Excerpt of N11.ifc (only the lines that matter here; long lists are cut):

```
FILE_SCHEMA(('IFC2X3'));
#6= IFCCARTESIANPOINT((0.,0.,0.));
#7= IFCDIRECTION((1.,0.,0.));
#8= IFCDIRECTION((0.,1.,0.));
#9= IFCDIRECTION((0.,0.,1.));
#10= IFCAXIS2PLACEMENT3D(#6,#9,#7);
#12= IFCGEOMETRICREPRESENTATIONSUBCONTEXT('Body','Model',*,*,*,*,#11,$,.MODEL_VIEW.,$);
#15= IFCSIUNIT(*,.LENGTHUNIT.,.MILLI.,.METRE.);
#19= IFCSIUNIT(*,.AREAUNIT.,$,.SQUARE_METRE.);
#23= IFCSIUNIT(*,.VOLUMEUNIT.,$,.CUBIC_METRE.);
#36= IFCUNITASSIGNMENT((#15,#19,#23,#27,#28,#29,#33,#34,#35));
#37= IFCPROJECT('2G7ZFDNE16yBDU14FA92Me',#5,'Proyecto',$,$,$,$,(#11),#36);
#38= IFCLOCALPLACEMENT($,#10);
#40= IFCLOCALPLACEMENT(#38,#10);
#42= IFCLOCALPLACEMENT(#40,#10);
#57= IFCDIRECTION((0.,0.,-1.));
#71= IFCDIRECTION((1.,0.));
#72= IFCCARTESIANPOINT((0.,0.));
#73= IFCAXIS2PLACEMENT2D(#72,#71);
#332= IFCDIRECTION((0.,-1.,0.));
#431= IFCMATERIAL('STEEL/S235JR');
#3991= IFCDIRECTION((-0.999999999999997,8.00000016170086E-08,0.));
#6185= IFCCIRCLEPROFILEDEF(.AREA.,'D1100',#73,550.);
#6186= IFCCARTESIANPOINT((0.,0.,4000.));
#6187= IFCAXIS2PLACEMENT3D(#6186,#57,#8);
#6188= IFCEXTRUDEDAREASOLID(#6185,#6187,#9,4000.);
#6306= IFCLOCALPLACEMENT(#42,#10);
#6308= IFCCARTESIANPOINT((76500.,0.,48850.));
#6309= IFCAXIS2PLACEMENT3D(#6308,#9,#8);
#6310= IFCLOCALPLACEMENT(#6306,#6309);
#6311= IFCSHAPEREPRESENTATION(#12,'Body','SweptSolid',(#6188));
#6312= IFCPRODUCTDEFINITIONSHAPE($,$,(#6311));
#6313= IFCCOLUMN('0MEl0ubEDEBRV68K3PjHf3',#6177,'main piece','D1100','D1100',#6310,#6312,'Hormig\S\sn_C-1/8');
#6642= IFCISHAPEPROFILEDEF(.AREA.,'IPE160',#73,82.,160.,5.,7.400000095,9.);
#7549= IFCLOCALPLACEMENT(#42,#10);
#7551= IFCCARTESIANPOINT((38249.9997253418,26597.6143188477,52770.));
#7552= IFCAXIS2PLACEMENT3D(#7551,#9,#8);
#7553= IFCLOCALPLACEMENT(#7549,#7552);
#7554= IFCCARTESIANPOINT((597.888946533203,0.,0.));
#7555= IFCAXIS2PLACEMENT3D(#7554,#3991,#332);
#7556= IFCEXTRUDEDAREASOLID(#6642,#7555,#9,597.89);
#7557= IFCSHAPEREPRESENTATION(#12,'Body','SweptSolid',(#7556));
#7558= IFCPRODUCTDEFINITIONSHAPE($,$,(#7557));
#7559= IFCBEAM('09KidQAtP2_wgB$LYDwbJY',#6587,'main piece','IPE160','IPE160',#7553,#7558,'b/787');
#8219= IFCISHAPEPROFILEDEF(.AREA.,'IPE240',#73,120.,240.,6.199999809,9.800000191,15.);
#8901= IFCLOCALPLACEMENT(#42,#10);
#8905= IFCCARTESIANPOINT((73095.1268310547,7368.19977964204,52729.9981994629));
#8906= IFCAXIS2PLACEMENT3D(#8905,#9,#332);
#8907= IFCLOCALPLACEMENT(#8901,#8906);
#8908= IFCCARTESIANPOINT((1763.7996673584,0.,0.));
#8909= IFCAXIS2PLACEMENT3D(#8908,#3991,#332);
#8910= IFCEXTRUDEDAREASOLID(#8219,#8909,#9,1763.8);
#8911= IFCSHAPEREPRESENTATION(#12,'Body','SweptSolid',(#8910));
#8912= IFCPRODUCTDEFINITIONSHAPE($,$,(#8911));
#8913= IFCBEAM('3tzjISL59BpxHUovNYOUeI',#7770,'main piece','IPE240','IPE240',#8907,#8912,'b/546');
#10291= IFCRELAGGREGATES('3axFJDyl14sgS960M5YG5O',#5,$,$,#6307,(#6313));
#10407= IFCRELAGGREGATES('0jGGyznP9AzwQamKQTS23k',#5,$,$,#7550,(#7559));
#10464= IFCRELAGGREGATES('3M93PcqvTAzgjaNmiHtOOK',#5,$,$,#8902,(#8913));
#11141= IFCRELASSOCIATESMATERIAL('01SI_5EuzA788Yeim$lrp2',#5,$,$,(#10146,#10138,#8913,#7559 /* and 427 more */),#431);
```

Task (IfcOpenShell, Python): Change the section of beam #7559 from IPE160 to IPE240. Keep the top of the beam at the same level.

```python
import ifcopenshell
import ifcopenshell.util.element
import ifcopenshell.util.representation

model = ifcopenshell.open("N11.ifc")

member = model.by_id(7559)
source = next(p for p in model.by_type("IfcIShapeProfileDef") if p.ProfileName == "IPE240")

body = ifcopenshell.util.representation.get_representation(member, "Model", "Body")
solid = body.Items[0]
old_profile = solid.SweptArea

# Copy the section's sizes but keep this member's own profile position.
profile = ifcopenshell.util.element.copy(model, source)
# Profiles are centred, so shift by half the change in depth to hold the top.
shift = (old_profile.OverallDepth - profile.OverallDepth) / 2
x, y = old_profile.Position.Location.Coordinates
up = (0.0, 1.0)  # upwards, in the solid's own plane
location = model.createIfcCartesianPoint((x + up[0] * shift, y + up[1] * shift))
profile.Position = model.createIfcAxis2Placement2D(location, old_profile.Position.RefDirection)
solid.SweptArea = profile
if not model.get_total_inverses(old_profile):
    ifcopenshell.util.element.remove_deep2(model, old_profile)
member.Description = member.Description.replace("IPE160", "IPE240")
member.ObjectType = member.ObjectType.replace("IPE160", "IPE240")

print(solid.SweptArea)

model.write("N11_updated.ifc")
```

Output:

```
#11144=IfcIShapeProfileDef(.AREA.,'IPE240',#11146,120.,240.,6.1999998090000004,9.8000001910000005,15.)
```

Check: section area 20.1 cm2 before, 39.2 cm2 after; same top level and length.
